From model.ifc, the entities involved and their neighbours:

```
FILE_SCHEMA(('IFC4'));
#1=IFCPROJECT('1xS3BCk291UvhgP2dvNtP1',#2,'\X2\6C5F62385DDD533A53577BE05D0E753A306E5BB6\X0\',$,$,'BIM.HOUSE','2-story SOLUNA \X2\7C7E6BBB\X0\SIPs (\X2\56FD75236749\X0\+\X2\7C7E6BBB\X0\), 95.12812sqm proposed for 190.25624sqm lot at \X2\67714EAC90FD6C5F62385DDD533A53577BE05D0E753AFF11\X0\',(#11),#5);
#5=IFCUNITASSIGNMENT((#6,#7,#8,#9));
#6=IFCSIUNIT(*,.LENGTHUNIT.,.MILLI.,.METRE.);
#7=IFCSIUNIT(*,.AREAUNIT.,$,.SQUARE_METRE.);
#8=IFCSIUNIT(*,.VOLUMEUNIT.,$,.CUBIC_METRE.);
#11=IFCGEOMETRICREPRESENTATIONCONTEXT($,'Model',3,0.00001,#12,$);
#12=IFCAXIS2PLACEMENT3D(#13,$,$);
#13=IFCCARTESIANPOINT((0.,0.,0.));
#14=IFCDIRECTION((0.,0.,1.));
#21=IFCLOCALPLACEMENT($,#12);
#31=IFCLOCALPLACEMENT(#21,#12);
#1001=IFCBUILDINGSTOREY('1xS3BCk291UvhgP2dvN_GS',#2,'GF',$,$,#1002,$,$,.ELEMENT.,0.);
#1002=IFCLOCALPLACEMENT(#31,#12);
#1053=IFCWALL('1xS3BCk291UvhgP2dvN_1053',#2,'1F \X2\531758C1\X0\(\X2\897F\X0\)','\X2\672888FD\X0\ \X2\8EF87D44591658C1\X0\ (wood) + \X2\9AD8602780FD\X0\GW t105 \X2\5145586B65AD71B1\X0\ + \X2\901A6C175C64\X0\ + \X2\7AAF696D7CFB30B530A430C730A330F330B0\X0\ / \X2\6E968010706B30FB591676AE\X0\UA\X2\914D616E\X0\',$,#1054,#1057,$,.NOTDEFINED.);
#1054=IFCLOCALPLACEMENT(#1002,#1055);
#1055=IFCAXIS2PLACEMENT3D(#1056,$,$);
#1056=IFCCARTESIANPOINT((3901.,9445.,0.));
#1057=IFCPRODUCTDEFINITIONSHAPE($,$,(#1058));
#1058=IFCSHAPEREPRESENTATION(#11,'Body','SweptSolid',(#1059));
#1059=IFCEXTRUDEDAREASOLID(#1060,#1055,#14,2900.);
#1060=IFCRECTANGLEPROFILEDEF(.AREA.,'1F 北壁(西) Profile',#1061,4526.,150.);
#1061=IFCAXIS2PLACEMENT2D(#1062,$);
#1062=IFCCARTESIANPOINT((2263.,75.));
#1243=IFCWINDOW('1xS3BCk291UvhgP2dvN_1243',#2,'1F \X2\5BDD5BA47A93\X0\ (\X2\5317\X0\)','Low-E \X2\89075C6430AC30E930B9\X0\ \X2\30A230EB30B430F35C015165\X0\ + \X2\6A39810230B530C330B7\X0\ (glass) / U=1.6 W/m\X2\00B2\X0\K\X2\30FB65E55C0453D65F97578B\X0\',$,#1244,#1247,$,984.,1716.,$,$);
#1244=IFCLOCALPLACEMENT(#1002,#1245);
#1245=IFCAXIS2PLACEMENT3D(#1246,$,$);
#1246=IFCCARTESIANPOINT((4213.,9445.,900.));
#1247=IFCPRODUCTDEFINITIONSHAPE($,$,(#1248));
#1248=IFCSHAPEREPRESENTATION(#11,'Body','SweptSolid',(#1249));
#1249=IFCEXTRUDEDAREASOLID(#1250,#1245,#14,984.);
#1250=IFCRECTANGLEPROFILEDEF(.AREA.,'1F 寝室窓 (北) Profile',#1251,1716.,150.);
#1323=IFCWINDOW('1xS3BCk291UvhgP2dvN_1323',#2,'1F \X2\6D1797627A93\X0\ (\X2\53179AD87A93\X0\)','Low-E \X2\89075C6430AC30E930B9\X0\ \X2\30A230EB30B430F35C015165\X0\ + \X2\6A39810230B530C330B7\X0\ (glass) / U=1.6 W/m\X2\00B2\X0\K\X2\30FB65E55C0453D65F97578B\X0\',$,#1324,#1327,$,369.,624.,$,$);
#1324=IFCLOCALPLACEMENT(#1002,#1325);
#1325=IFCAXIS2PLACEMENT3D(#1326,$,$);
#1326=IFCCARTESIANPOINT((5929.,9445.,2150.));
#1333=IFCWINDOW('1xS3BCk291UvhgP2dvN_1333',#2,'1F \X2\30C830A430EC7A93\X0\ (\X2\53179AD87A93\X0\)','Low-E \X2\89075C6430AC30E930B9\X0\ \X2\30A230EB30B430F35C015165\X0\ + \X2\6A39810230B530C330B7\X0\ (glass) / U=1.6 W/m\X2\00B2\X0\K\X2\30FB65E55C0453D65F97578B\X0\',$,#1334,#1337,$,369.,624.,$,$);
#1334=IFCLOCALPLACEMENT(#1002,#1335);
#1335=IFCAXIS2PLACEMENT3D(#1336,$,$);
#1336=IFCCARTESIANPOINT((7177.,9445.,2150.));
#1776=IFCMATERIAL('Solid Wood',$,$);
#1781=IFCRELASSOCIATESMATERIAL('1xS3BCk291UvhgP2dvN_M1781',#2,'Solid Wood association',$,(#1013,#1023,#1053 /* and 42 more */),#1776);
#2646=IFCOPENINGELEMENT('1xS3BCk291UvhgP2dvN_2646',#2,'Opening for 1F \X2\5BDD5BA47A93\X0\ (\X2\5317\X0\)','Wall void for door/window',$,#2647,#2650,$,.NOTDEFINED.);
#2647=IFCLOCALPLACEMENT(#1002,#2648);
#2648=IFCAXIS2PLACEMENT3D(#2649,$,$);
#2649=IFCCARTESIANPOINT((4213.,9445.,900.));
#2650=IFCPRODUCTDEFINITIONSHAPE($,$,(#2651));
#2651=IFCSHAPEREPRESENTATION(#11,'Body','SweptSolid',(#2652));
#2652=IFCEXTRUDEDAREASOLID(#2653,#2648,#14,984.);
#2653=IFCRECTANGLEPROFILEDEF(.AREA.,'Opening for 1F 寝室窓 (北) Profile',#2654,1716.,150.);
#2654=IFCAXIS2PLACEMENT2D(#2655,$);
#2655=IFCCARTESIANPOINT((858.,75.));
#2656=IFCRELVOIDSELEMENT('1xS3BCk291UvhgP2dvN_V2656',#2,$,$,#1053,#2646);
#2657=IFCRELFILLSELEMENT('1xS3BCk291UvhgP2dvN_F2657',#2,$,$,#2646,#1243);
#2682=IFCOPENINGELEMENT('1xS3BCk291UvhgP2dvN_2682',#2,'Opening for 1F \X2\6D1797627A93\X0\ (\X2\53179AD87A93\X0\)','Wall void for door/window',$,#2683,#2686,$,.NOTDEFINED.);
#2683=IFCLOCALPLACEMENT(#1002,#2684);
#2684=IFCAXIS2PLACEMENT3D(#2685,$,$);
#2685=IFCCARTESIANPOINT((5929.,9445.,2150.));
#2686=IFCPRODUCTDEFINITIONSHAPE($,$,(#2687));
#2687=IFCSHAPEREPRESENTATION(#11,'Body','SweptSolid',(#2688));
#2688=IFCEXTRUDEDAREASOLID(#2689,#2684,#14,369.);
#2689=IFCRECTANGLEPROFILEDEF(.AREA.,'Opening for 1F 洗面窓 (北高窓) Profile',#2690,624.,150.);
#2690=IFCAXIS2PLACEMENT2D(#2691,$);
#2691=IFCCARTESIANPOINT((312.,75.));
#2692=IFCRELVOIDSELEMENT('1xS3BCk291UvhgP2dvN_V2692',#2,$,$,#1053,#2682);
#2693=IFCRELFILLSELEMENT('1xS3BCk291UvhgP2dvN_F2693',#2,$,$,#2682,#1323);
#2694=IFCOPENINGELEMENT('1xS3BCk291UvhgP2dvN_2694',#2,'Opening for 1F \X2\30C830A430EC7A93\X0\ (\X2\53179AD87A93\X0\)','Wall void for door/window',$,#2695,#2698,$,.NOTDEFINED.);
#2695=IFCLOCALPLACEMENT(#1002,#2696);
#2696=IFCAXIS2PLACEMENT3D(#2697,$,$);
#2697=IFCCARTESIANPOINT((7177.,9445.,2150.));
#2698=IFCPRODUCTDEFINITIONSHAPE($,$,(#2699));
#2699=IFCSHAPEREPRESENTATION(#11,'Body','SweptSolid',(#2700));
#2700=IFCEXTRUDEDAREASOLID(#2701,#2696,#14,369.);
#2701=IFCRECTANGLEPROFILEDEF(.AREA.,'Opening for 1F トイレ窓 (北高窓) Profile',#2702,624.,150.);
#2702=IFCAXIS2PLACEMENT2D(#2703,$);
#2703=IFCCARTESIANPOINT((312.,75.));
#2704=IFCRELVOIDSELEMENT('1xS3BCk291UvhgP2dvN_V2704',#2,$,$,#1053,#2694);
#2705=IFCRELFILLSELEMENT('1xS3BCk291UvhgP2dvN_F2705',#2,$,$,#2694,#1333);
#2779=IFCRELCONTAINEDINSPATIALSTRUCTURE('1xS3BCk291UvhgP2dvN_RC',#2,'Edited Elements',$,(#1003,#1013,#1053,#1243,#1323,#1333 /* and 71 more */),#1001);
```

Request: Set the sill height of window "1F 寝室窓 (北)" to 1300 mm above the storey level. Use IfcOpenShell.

```python
import numpy as np
import ifcopenshell
import ifcopenshell.api.geometry
import ifcopenshell.geom
import ifcopenshell.util.element
import ifcopenshell.util.placement
import ifcopenshell.util.shape
import ifcopenshell.util.unit

model = ifcopenshell.open("model.ifc")
unit_scale = ifcopenshell.util.unit.calculate_unit_scale(model)

window = model.by_id(1243)
opening = window.FillsVoids[0].RelatingOpeningElement
storey = ifcopenshell.util.element.get_container(window, ifc_class="IfcBuildingStorey")
level = ifcopenshell.util.placement.get_local_placement(storey.ObjectPlacement)[2, 3]

# The opening's origin need not be at the sill, so measure its lowest point.
shape = ifcopenshell.geom.create_shape(ifcopenshell.geom.settings(), opening)
bottom = ifcopenshell.util.shape.get_shape_bottom_elevation(shape, shape.geometry) / unit_scale
dz = level + 1.3 / unit_scale - bottom

shift = np.array([0.0, 0.0, dz])
# The window is not placed relative to its opening, so move both.
for product in (opening, window):
    matrix = ifcopenshell.util.placement.get_local_placement(product.ObjectPlacement)
    matrix[:3, 3] += shift
    ifcopenshell.api.geometry.edit_object_placement(model, product=product, matrix=matrix, is_si=False)

print(f"moved by {dz * unit_scale:+.3f} m")

model.write("model_v2.ifc")
```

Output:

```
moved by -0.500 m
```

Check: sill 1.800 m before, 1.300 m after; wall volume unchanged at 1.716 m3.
